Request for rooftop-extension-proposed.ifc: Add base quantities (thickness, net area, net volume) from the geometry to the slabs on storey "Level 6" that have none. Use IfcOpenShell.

First a look at what the model holds.

```python
import ifcopenshell
import ifcopenshell.util.element
import ifcopenshell.util.unit

model = ifcopenshell.open("rooftop-extension-proposed.ifc")
print(model.schema)
for unit_type in ("LENGTHUNIT", "AREAUNIT", "VOLUMEUNIT"):
    print(unit_type, ifcopenshell.util.unit.calculate_unit_scale(model, unit_type))
storey = next(s for s in model.by_type("IfcBuildingStorey") if s.Name == "Level 6")
slabs = [e for e in ifcopenshell.util.element.get_decomposition(storey) if e.is_a("IfcSlab")]
for e in sorted(slabs, key=lambda e: e.id()):
    print(e.id(), e.is_a(), e.Name, list(ifcopenshell.util.element.get_psets(e, qtos_only=True)), sep=" | ")
```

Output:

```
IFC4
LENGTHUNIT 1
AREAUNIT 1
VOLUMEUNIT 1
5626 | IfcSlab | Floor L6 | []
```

```python
import ifcopenshell
import ifcopenshell.api.pset
import ifcopenshell.geom
import ifcopenshell.util.element
import ifcopenshell.util.shape
import ifcopenshell.util.unit

model = ifcopenshell.open("rooftop-extension-proposed.ifc")
unit_scale = ifcopenshell.util.unit.calculate_unit_scale(model)
area_scale = ifcopenshell.util.unit.calculate_unit_scale(model, "AREAUNIT")
volume_scale = ifcopenshell.util.unit.calculate_unit_scale(model, "VOLUMEUNIT")
settings = ifcopenshell.geom.settings()

storey = next(s for s in model.by_type("IfcBuildingStorey") if s.Name == "Level 6")
slabs = [e for e in ifcopenshell.util.element.get_decomposition(storey) if e.is_a("IfcSlab")]

for e in sorted(slabs, key=lambda e: e.id()):
    if ifcopenshell.util.element.get_psets(e, qtos_only=True, should_inherit=False):
        continue
    # Geometry comes back in metres, in the element's own axes.
    shape = ifcopenshell.geom.create_shape(settings, e)
    values = {
        "Width": ifcopenshell.util.shape.get_z(shape.geometry) / unit_scale,
        "NetArea": ifcopenshell.util.shape.get_footprint_area(shape.geometry) / area_scale,
        "NetVolume": ifcopenshell.util.shape.get_volume(shape.geometry) / volume_scale,
    }
    qto = ifcopenshell.api.pset.add_qto(model, product=e, name="Qto_SlabBaseQuantities")
    ifcopenshell.api.pset.edit_qto(model, qto=qto, properties=values)
    print(e.id(), {k: round(v, 3) for k, v in values.items()})

model.write("rooftop-extension-proposed_v2.ifc")
```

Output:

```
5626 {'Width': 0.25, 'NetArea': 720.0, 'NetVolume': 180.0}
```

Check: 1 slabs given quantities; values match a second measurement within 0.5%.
